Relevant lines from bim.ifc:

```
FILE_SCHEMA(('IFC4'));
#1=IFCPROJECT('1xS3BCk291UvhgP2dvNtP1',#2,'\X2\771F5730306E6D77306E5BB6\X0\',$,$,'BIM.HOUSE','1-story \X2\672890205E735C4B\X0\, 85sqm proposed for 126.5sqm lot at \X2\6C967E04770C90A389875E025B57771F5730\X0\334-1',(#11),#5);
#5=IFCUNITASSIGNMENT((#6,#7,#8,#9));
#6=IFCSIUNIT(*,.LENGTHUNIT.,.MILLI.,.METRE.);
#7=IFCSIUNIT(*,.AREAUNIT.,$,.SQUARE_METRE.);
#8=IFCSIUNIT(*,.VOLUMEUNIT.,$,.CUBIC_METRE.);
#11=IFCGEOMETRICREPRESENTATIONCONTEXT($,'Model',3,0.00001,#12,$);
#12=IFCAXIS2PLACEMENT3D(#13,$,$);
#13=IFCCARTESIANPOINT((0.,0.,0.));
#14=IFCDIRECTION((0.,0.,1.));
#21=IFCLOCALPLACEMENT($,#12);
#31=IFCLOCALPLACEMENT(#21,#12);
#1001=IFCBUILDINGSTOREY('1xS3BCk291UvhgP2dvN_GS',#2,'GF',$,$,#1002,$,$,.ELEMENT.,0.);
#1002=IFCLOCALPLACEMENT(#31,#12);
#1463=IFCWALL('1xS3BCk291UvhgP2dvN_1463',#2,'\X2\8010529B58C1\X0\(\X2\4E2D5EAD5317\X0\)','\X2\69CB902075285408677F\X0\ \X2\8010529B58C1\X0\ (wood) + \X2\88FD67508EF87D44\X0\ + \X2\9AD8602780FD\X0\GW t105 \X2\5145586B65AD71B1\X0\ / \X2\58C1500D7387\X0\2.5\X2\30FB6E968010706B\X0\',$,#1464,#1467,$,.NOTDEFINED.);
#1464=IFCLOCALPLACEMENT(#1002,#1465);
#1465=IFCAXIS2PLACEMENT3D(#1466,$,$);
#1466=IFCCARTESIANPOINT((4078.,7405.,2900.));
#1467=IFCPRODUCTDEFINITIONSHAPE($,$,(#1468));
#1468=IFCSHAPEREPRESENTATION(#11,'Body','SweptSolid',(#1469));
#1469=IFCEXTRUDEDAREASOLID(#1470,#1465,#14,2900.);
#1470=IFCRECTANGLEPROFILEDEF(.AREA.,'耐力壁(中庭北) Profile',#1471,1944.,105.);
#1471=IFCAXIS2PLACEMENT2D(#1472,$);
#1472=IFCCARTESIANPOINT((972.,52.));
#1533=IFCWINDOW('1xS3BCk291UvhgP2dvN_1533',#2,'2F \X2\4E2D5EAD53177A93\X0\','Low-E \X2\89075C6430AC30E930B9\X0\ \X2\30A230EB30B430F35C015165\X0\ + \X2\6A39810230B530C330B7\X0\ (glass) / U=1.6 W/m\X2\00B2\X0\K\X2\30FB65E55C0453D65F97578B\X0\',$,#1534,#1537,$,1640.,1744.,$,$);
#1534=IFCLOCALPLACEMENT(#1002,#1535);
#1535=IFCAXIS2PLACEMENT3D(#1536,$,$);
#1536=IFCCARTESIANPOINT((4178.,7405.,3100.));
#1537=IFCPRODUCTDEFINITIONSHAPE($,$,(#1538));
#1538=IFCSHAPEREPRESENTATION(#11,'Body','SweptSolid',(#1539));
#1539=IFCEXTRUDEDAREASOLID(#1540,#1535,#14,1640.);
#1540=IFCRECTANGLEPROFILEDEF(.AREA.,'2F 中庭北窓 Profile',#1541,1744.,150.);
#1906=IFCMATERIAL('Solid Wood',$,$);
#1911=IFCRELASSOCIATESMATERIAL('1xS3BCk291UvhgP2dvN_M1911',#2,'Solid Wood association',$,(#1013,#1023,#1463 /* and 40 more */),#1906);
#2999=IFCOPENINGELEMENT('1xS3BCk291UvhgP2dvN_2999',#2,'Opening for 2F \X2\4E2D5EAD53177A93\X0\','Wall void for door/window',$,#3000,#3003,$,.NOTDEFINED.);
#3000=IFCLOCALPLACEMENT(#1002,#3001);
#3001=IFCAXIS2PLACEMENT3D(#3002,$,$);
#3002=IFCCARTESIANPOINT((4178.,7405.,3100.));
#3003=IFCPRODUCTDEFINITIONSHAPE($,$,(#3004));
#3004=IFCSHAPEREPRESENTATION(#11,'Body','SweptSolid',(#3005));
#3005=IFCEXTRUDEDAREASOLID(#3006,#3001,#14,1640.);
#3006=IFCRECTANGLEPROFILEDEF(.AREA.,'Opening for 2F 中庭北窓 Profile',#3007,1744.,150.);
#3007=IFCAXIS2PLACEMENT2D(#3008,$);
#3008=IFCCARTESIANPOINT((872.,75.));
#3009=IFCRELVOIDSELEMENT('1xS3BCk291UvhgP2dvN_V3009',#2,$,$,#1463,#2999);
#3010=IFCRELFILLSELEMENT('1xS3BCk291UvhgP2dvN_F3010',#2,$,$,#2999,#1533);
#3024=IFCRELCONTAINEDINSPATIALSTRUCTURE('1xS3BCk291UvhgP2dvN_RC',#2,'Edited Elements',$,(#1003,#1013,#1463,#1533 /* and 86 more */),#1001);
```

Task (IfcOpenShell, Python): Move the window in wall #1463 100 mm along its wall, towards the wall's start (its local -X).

```python
import ifcopenshell
import ifcopenshell.api.geometry
import ifcopenshell.util.placement
import ifcopenshell.util.unit

model = ifcopenshell.open("bim.ifc")
unit_scale = ifcopenshell.util.unit.calculate_unit_scale(model)

window = model.by_guid("1xS3BCk291UvhgP2dvN_1533")
opening = window.FillsVoids[0].RelatingOpeningElement
wall = opening.VoidsElements[0].RelatingBuildingElement

wall_matrix = ifcopenshell.util.placement.get_local_placement(wall.ObjectPlacement)
shift = wall_matrix[:3, 0] * -0.1 / unit_scale
before = ifcopenshell.util.placement.get_local_placement(window.ObjectPlacement)[:3, 3].copy()

# The window is not placed relative to its opening, so move both.
for product in (opening, window):
    matrix = ifcopenshell.util.placement.get_local_placement(product.ObjectPlacement)
    matrix[:3, 3] += shift
    ifcopenshell.api.geometry.edit_object_placement(model, product=product, matrix=matrix, is_si=False)

after = ifcopenshell.util.placement.get_local_placement(window.ObjectPlacement)[:3, 3]
print("window moved by", (after - before).round(3) + 0.0)

model.write("bim_v2.ifc")
```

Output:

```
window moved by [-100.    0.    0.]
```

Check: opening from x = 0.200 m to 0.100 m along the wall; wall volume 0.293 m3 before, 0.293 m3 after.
